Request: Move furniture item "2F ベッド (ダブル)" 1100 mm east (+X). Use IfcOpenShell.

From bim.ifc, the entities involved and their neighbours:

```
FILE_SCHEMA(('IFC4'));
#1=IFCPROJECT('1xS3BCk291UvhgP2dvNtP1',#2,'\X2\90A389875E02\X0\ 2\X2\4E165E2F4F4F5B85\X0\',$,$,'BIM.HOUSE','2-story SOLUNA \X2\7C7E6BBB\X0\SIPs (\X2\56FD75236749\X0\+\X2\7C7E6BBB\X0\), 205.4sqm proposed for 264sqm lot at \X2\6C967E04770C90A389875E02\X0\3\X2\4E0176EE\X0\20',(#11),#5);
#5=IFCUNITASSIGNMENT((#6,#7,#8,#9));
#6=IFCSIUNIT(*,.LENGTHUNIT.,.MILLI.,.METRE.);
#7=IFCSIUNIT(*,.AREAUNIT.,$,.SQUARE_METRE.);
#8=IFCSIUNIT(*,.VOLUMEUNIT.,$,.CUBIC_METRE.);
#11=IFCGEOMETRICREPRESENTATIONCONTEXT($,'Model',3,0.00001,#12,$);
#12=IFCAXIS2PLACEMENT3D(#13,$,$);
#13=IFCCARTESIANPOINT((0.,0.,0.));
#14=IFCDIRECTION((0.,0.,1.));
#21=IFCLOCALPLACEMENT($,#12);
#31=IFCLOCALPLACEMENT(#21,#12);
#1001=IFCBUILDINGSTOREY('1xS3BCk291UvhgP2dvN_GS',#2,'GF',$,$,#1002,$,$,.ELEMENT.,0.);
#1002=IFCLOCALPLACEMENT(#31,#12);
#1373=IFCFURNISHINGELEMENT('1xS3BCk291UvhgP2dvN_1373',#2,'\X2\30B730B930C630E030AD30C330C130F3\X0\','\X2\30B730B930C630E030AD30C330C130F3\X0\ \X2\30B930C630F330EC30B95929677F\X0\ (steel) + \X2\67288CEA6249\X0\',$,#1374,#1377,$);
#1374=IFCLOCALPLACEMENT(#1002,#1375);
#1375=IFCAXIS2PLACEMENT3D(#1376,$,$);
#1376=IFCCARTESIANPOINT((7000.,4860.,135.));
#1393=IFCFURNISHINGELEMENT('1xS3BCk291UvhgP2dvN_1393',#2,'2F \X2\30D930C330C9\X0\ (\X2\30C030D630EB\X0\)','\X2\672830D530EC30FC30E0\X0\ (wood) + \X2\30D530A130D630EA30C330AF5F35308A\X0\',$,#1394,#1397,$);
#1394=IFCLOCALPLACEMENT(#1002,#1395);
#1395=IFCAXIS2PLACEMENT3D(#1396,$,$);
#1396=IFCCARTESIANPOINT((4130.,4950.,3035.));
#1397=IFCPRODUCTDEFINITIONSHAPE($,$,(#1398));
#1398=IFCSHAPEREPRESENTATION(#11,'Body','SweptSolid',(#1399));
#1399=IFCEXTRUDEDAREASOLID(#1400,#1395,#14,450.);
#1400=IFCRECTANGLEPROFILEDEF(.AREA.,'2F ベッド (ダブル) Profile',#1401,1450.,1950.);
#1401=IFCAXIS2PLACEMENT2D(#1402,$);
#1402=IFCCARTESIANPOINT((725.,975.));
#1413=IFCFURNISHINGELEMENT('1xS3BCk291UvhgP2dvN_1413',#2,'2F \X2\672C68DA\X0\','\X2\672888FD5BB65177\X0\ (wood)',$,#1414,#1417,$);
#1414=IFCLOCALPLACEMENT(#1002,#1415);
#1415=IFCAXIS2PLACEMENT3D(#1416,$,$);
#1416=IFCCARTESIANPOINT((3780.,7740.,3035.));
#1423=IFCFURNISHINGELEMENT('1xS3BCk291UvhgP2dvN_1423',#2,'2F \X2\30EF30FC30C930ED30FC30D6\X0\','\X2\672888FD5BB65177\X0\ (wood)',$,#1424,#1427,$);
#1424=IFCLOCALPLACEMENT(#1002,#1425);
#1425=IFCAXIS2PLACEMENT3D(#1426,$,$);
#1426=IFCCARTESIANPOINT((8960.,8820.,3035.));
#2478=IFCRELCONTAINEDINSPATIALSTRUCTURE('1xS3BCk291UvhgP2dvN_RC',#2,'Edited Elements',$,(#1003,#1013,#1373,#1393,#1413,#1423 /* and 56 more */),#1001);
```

```python
import ifcopenshell
import ifcopenshell.api.geometry
import ifcopenshell.util.placement
import ifcopenshell.util.unit

model = ifcopenshell.open("bim.ifc")
unit_scale = ifcopenshell.util.unit.calculate_unit_scale(model)

item = model.by_guid("1xS3BCk291UvhgP2dvN_1393")
matrix = ifcopenshell.util.placement.get_local_placement(item.ObjectPlacement)
matrix[0, 3] += 1.1 / unit_scale
ifcopenshell.api.geometry.edit_object_placement(model, product=item, matrix=matrix, is_si=False)

print(ifcopenshell.util.placement.get_local_placement(item.ObjectPlacement).round(3) + 0.0)

model.write("bim_updated.ifc")
```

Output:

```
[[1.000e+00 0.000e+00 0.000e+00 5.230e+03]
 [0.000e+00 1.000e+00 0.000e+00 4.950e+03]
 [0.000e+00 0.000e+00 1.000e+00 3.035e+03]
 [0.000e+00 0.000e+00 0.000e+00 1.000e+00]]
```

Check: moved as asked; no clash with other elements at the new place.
